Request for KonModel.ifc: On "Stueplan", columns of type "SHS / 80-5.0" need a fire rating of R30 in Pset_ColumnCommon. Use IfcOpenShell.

First a look at what the model holds.

```python
import ifcopenshell
import ifcopenshell.util.element

model = ifcopenshell.open("KonModel.ifc")
print(model.schema)
storey = next(s for s in model.by_type("IfcBuildingStorey") if s.Name == "Stueplan")
columns = [e for e in ifcopenshell.util.element.get_decomposition(storey) if e.is_a("IfcColumn")]
seen = {}
for e in columns:
    element_type = ifcopenshell.util.element.get_type(e)
    key = (element_type.Name if element_type != e and element_type else None, ifcopenshell.util.element.get_pset(e, "Pset_ColumnCommon", "FireRating"))
    seen[key] = seen.get(key, 0) + 1
for (name, value), count in sorted(seen.items(), key=str):
    print(count, "x", name, "|", value)
```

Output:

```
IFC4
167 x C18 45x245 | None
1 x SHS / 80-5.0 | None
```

```python
import ifcopenshell
import ifcopenshell.api.pset
import ifcopenshell.util.element

model = ifcopenshell.open("KonModel.ifc")

storey = next(s for s in model.by_type("IfcBuildingStorey") if s.Name == "Stueplan")
columns = [e for e in ifcopenshell.util.element.get_decomposition(storey) if e.is_a("IfcColumn")]

count = 0
for e in columns:
    element_type = ifcopenshell.util.element.get_type(e)
    if element_type in (None, e) or element_type.Name != "SHS / 80-5.0":
        continue
    # add_pset returns the element's existing set when there is one.
    pset = ifcopenshell.api.pset.add_pset(model, product=e, name="Pset_ColumnCommon")
    ifcopenshell.api.pset.edit_pset(model, pset=pset, properties={"FireRating": "R30"})
    count += 1

print(count, "columns updated")

model.write("KonModel_v2.ifc")
```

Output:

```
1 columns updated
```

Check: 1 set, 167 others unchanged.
